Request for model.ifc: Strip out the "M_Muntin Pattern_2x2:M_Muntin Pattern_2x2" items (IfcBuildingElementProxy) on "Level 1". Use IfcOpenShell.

First a look at what the model holds.

```python
import ifcopenshell
import ifcopenshell.util.element

model = ifcopenshell.open("model.ifc")
print(model.schema)
storey = next(s for s in model.by_type("IfcBuildingStorey") if s.Name == "Level 1")
proxies = [e for e in ifcopenshell.util.element.get_decomposition(storey) if e.is_a("IfcBuildingElementProxy")]
seen = {}
for e in proxies:
    element_type = ifcopenshell.util.element.get_type(e)
    name = element_type.Name if element_type not in (None, e) else None
    seen[name] = seen.get(name, 0) + 1
for name, count in sorted(seen.items(), key=str):
    print(count, "x", name)
```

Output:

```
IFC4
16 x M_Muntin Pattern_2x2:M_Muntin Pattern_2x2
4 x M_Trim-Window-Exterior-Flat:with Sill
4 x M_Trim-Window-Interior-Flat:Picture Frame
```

```python
import ifcopenshell
import ifcopenshell.api.root
import ifcopenshell.util.element

model = ifcopenshell.open("model.ifc")

storey = next(s for s in model.by_type("IfcBuildingStorey") if s.Name == "Level 1")
proxies = [e for e in ifcopenshell.util.element.get_decomposition(storey) if e.is_a("IfcBuildingElementProxy")]
targets = [e for e in proxies if (t := ifcopenshell.util.element.get_type(e)) not in (None, e) and t.Name == "M_Muntin Pattern_2x2:M_Muntin Pattern_2x2"]

for e in targets:
    ifcopenshell.api.root.remove_product(model, product=e)
print(len(targets), "removed")

model.write("model-out.ifc")
```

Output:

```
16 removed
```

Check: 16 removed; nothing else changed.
